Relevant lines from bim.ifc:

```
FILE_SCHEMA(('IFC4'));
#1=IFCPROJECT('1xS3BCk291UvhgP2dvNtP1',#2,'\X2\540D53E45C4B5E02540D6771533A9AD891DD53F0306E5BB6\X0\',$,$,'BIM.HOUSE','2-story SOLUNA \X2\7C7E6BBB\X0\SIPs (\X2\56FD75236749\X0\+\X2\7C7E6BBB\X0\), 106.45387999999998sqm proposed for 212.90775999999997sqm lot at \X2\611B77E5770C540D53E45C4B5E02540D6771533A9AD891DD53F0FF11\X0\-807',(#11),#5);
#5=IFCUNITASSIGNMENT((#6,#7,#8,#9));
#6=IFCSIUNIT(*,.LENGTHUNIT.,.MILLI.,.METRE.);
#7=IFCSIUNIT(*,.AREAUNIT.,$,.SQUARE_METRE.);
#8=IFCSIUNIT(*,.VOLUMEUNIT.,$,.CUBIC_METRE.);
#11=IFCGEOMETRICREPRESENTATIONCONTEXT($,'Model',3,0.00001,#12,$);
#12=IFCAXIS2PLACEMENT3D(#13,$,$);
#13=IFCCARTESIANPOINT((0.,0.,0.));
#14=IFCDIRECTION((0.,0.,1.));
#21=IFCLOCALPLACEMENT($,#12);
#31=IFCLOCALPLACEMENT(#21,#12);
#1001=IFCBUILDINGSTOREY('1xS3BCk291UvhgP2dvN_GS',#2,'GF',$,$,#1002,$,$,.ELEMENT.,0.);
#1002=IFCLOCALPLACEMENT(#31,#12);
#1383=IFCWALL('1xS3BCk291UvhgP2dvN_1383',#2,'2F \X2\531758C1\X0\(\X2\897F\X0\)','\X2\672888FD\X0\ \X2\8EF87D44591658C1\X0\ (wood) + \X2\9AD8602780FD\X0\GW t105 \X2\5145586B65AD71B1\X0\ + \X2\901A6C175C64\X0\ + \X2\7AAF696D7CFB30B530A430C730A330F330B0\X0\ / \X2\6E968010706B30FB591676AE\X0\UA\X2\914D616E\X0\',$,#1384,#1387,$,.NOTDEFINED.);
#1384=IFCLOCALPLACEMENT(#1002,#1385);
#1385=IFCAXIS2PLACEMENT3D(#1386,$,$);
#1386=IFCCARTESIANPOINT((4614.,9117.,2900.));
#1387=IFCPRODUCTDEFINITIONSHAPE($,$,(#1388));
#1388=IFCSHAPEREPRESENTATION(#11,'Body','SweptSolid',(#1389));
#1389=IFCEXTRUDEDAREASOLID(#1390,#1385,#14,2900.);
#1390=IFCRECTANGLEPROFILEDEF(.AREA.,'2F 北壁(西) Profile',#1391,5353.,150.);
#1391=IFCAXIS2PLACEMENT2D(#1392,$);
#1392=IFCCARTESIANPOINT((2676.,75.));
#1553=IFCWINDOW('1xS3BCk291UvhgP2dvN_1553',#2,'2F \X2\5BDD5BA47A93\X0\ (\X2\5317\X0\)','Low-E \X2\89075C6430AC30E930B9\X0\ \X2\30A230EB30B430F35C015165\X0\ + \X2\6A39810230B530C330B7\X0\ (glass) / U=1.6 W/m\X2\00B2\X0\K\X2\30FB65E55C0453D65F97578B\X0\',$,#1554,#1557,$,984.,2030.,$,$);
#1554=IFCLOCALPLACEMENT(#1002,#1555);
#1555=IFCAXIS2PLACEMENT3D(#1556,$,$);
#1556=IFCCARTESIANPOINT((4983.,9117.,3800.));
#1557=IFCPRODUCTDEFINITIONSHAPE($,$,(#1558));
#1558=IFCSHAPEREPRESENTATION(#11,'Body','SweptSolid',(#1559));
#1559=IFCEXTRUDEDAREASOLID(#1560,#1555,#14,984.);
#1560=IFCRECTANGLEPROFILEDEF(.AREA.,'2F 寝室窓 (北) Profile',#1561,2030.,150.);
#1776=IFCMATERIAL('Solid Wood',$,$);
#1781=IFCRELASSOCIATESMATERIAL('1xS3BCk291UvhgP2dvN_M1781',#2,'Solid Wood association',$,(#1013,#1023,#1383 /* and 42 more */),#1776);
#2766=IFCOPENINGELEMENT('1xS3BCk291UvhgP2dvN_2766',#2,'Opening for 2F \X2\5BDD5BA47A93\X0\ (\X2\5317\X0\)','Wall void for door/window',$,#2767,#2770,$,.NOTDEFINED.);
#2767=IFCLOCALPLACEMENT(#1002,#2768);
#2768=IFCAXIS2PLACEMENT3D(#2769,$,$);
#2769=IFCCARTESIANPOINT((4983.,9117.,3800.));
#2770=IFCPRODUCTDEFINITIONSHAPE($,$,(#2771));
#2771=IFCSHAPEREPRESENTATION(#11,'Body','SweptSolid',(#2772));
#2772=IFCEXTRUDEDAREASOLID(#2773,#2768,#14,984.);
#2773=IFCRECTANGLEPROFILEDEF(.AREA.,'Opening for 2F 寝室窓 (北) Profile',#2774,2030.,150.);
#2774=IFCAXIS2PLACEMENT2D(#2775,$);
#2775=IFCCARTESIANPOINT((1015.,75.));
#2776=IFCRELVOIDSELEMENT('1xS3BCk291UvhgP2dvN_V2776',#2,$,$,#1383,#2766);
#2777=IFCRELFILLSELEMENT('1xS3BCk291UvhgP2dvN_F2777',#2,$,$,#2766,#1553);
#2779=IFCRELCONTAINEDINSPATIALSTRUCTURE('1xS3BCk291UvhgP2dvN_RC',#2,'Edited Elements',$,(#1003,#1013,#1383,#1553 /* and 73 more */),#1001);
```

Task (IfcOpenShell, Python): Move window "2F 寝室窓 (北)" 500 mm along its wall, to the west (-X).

```python
import ifcopenshell
import ifcopenshell.api.geometry
import ifcopenshell.util.placement
import ifcopenshell.util.unit

model = ifcopenshell.open("bim.ifc")
unit_scale = ifcopenshell.util.unit.calculate_unit_scale(model)

window = model.by_guid("1xS3BCk291UvhgP2dvN_1553")
opening = window.FillsVoids[0].RelatingOpeningElement
wall = opening.VoidsElements[0].RelatingBuildingElement

wall_matrix = ifcopenshell.util.placement.get_local_placement(wall.ObjectPlacement)
shift = wall_matrix[:3, 0] * -0.5 / unit_scale
before = ifcopenshell.util.placement.get_local_placement(window.ObjectPlacement)[:3, 3].copy()

# The window is not placed relative to its opening, so move both.
for product in (opening, window):
    matrix = ifcopenshell.util.placement.get_local_placement(product.ObjectPlacement)
    matrix[:3, 3] += shift
    ifcopenshell.api.geometry.edit_object_placement(model, product=product, matrix=matrix, is_si=False)

after = ifcopenshell.util.placement.get_local_placement(window.ObjectPlacement)[:3, 3]
print("window moved by", (after - before).round(3) + 0.0)

model.write("bim_rev.ifc")
```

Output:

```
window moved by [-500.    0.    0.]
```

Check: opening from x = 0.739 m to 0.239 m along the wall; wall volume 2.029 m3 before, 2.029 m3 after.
